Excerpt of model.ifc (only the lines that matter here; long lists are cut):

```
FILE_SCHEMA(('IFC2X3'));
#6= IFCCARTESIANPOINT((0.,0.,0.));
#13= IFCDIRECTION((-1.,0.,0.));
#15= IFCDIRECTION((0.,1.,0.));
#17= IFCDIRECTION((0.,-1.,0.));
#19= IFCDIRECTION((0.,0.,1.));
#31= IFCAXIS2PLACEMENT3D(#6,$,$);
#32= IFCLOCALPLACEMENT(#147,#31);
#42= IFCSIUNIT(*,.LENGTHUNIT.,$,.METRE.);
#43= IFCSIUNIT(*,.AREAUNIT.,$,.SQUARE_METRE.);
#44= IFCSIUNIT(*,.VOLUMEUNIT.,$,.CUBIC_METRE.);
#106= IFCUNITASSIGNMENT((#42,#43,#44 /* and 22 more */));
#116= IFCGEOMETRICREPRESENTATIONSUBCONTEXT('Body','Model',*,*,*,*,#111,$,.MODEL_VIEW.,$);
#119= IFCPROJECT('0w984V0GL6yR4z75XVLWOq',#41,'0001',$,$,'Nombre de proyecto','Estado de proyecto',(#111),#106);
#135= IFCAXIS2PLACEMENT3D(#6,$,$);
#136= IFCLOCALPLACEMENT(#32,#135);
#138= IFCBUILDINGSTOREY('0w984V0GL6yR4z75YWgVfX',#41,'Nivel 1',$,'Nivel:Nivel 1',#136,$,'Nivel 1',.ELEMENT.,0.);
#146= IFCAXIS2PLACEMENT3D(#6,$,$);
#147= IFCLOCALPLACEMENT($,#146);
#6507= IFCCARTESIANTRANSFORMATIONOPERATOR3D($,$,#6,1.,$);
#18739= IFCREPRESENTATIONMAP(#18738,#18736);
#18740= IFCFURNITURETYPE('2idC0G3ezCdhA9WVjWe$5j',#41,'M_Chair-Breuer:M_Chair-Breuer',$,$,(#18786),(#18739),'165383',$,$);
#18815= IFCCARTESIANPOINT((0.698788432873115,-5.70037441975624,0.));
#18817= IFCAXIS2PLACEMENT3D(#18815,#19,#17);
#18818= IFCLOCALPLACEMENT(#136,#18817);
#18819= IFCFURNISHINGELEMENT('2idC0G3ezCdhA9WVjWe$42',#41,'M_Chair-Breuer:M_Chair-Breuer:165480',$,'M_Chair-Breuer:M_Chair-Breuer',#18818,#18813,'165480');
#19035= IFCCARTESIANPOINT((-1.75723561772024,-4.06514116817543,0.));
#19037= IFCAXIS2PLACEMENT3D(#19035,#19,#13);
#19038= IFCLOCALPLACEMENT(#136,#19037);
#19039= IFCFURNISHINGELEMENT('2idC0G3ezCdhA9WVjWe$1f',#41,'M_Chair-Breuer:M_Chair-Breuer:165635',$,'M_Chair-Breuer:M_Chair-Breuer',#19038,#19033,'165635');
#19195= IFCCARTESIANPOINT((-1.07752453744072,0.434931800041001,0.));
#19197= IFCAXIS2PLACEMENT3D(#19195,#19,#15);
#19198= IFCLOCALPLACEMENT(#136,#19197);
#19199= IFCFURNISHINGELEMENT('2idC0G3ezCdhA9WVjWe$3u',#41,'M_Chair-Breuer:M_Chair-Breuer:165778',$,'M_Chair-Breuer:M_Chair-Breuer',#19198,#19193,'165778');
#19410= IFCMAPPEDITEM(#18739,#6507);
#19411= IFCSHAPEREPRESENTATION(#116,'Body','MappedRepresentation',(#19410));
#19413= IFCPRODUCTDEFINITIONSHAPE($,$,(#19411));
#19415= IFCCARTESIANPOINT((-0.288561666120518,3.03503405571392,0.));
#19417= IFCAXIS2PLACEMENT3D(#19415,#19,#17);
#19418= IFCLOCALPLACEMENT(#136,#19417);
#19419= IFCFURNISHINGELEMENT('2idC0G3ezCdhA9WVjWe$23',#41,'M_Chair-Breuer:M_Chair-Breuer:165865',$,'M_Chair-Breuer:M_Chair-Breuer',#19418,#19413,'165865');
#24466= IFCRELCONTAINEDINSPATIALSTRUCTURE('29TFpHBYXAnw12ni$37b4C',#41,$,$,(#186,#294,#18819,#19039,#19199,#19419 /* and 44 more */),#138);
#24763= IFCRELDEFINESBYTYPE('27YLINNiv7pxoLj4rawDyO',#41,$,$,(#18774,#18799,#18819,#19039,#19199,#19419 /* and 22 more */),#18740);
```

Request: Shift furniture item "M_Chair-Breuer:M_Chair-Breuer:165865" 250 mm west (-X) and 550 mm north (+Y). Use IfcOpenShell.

```python
import ifcopenshell
import ifcopenshell.api.geometry
import ifcopenshell.util.placement

model = ifcopenshell.open("model.ifc")

item = model.by_id(19419)
matrix = ifcopenshell.util.placement.get_local_placement(item.ObjectPlacement)
matrix[0, 3] -= 0.25
matrix[1, 3] += 0.55
ifcopenshell.api.geometry.edit_object_placement(model, product=item, matrix=matrix, is_si=False)

print(ifcopenshell.util.placement.get_local_placement(item.ObjectPlacement).round(3) + 0.0)

model.write("model-out.ifc")
```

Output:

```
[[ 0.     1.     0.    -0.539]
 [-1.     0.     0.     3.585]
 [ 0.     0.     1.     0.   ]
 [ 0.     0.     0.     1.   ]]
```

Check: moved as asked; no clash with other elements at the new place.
